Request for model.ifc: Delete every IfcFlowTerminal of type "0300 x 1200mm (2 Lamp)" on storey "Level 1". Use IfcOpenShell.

First a look at what the model holds.

```python
import ifcopenshell
import ifcopenshell.util.element

model = ifcopenshell.open("model.ifc")
print(model.schema)
storey = next(s for s in model.by_type("IfcBuildingStorey") if s.Name == "Level 1")
terminals = [e for e in ifcopenshell.util.element.get_decomposition(storey) if e.is_a("IfcFlowTerminal")]
seen = {}
for e in terminals:
    element_type = ifcopenshell.util.element.get_type(e)
    name = element_type.Name if element_type not in (None, e) else None
    seen[name] = seen.get(name, 0) + 1
for name, count in sorted(seen.items(), key=str):
    print(count, "x", name)
```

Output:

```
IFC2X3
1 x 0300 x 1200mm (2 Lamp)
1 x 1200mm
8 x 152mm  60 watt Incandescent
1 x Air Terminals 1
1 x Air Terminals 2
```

```python
import ifcopenshell
import ifcopenshell.api.root
import ifcopenshell.util.element

model = ifcopenshell.open("model.ifc")

storey = next(s for s in model.by_type("IfcBuildingStorey") if s.Name == "Level 1")
terminals = [e for e in ifcopenshell.util.element.get_decomposition(storey) if e.is_a("IfcFlowTerminal")]
targets = [e for e in terminals if (t := ifcopenshell.util.element.get_type(e)) not in (None, e) and t.Name == "0300 x 1200mm (2 Lamp)"]

for e in targets:
    ifcopenshell.api.root.remove_product(model, product=e)
print(len(targets), "removed")

model.write("model_edited.ifc")
```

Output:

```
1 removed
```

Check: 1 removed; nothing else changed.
